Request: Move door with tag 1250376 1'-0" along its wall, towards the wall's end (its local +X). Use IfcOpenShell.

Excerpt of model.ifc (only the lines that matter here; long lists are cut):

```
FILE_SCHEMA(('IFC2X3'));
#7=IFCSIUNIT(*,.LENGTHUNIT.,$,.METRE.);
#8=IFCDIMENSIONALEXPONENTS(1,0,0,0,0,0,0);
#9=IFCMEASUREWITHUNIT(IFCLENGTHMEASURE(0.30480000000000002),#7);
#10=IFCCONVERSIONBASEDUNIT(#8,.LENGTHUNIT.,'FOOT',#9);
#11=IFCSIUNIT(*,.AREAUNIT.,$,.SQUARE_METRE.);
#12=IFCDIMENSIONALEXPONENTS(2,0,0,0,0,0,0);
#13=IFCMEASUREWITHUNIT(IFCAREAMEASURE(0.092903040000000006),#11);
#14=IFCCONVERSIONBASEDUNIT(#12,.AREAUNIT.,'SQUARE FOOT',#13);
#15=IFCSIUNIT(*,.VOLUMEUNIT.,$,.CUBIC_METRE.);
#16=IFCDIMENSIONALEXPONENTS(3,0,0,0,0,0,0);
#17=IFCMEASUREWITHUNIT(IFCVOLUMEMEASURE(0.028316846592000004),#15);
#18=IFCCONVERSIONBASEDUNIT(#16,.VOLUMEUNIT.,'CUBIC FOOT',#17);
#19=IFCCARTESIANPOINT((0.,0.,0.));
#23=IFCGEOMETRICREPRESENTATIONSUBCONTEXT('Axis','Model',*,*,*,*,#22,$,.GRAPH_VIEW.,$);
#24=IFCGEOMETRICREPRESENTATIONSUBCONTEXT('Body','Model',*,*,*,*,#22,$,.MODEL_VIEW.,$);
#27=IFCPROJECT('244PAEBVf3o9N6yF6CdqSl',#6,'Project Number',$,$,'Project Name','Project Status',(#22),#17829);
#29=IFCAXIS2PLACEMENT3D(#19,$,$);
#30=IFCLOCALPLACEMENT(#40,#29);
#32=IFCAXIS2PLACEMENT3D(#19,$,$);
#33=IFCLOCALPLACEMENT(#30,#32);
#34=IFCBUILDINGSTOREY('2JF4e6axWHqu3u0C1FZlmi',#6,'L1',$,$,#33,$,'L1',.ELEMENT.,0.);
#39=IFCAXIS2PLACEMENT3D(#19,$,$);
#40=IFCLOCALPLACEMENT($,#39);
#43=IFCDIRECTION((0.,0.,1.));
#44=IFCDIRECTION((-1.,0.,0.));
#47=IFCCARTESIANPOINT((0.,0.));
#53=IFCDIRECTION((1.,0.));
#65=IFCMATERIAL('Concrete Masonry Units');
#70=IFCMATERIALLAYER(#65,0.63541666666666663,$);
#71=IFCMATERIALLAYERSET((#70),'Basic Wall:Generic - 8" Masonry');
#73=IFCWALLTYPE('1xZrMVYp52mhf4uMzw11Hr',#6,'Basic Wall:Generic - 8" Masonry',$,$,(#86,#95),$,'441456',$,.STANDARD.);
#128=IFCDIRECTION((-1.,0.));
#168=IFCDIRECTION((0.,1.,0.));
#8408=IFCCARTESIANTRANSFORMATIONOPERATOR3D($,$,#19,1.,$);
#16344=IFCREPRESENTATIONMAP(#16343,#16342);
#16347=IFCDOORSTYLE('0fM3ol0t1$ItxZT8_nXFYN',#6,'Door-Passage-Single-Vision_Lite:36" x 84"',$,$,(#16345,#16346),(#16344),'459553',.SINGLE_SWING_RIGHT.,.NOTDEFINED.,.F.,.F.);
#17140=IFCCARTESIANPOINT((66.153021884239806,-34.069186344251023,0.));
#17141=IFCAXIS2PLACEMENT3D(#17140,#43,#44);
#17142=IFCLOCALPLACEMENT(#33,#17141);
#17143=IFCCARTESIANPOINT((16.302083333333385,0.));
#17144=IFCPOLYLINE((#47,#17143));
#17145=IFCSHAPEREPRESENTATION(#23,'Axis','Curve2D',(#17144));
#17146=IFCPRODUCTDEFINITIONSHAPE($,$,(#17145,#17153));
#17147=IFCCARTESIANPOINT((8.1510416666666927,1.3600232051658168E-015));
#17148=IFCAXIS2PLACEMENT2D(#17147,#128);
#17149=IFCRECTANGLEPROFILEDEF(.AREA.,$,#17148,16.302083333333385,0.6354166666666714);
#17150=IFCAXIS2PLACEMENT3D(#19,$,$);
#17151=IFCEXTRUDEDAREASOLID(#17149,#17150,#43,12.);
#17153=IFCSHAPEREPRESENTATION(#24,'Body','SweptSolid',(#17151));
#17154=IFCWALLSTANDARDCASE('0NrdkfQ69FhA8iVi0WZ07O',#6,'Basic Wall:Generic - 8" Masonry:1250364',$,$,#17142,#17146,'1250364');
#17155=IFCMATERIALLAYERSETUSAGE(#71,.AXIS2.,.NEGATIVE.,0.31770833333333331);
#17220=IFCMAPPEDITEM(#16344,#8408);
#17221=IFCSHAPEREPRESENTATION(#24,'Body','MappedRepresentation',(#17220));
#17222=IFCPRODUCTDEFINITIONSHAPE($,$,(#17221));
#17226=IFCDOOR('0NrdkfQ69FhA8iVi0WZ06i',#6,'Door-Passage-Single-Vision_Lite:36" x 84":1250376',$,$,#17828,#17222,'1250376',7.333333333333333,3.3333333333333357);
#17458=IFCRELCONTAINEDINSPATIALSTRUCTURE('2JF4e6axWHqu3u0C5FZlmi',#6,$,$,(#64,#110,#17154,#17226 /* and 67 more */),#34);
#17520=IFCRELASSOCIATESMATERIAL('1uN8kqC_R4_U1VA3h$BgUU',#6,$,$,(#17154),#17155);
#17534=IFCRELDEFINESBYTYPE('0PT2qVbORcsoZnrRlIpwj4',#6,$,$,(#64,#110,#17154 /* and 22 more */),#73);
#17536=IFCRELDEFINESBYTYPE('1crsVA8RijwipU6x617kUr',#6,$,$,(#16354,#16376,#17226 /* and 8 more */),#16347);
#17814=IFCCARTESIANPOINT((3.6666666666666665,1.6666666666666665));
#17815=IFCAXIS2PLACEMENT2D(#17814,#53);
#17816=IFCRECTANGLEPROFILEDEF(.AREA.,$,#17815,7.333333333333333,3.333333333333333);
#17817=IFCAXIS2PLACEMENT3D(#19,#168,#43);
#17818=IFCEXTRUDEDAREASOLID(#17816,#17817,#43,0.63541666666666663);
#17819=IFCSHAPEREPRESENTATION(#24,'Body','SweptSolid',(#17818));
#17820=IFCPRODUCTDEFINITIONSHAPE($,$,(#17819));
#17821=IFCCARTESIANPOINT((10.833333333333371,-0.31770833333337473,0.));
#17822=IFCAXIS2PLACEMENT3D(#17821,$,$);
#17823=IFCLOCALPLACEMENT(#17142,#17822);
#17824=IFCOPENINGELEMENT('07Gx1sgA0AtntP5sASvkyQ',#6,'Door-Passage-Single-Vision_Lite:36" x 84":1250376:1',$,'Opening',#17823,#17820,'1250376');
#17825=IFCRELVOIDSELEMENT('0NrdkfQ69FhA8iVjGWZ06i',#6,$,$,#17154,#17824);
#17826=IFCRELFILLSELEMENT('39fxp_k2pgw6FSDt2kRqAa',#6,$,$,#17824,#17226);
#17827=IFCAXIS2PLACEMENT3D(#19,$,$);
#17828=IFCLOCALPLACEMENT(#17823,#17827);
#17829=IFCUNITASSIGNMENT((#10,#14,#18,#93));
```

```python
import ifcopenshell
import ifcopenshell.api.geometry
import ifcopenshell.util.placement
import ifcopenshell.util.unit

model = ifcopenshell.open("model.ifc")
unit_scale = ifcopenshell.util.unit.calculate_unit_scale(model)

door = model.by_guid("0NrdkfQ69FhA8iVi0WZ06i")
opening = door.FillsVoids[0].RelatingOpeningElement
wall = opening.VoidsElements[0].RelatingBuildingElement

wall_matrix = ifcopenshell.util.placement.get_local_placement(wall.ObjectPlacement)
shift = wall_matrix[:3, 0] * 12 * 0.0254 / unit_scale
before = ifcopenshell.util.placement.get_local_placement(door.ObjectPlacement)[:3, 3].copy()

# The door is placed relative to its opening, so it follows when the opening moves.
matrix = ifcopenshell.util.placement.get_local_placement(opening.ObjectPlacement)
matrix[:3, 3] += shift
ifcopenshell.api.geometry.edit_object_placement(
    model, product=opening, matrix=matrix, is_si=False, should_transform_children=True
)

after = ifcopenshell.util.placement.get_local_placement(door.ObjectPlacement)[:3, 3]
print("door moved by", (after - before).round(3) + 0.0)

model.write("model_edited.ifc")
```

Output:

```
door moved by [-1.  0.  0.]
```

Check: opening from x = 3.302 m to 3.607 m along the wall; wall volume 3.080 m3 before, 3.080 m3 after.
